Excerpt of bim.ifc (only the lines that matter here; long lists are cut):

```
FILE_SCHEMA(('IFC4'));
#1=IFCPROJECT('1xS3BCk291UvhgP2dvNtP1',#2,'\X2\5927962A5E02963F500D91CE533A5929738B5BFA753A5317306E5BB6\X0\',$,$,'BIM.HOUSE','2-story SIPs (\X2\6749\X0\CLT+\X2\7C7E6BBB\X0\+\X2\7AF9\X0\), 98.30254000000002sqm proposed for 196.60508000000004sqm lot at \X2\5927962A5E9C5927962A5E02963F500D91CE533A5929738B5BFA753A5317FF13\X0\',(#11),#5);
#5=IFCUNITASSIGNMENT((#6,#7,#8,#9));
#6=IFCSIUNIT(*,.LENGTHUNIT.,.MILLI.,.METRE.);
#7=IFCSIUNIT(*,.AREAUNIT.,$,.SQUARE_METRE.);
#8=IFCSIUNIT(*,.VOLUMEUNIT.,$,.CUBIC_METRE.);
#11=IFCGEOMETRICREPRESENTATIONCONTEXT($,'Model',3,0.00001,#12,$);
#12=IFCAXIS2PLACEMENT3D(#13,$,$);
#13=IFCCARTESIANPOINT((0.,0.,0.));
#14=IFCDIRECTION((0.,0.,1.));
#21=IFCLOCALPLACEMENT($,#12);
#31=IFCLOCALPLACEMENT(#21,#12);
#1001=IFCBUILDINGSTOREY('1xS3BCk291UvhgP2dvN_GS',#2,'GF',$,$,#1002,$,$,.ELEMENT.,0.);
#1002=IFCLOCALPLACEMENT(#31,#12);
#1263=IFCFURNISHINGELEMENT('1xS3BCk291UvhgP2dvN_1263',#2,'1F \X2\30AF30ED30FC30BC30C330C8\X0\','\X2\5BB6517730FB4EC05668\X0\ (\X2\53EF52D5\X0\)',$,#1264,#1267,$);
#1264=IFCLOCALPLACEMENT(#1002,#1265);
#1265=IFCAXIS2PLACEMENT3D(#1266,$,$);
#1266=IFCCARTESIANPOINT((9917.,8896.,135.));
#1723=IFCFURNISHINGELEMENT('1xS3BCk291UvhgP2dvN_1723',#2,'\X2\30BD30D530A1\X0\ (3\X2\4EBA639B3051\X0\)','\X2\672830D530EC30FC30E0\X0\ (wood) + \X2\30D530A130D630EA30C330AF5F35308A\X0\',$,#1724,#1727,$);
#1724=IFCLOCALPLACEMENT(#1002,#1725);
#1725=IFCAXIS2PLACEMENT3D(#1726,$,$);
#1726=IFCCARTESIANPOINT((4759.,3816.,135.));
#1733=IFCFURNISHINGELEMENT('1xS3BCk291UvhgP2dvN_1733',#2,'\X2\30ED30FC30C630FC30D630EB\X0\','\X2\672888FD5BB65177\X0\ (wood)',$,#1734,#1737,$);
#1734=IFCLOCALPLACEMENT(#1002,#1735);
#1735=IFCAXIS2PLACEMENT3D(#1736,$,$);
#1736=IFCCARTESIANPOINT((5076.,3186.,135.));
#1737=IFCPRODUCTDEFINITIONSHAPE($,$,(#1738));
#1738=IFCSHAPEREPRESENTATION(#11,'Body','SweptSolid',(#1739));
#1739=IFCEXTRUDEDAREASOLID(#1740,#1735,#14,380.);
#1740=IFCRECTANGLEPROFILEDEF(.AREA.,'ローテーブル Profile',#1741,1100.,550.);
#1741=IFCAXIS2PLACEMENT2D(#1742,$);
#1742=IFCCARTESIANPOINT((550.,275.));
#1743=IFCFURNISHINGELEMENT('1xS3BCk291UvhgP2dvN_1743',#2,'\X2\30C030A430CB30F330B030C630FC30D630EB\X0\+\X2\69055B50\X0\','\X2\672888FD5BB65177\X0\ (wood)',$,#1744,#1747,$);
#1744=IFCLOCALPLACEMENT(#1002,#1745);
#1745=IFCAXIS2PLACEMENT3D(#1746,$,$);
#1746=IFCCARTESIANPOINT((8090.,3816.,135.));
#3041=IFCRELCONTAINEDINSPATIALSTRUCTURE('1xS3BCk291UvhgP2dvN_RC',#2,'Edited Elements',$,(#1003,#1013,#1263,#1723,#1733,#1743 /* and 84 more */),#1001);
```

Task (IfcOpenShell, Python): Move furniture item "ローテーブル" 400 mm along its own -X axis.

```python
import ifcopenshell
import ifcopenshell.api.geometry
import ifcopenshell.util.placement

model = ifcopenshell.open("bim.ifc")

item = model.by_guid("1xS3BCk291UvhgP2dvN_1733")
matrix = ifcopenshell.util.placement.get_local_placement(item.ObjectPlacement)
matrix[:3, 3] -= matrix[:3, 0] * 400.0
ifcopenshell.api.geometry.edit_object_placement(model, product=item, matrix=matrix, is_si=False)

print(ifcopenshell.util.placement.get_local_placement(item.ObjectPlacement).round(3) + 0.0)

model.write("bim_updated.ifc")
```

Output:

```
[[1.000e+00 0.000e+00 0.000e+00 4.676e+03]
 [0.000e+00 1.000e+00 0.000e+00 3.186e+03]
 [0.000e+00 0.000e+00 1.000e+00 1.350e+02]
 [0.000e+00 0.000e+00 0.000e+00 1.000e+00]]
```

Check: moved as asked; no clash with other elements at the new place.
